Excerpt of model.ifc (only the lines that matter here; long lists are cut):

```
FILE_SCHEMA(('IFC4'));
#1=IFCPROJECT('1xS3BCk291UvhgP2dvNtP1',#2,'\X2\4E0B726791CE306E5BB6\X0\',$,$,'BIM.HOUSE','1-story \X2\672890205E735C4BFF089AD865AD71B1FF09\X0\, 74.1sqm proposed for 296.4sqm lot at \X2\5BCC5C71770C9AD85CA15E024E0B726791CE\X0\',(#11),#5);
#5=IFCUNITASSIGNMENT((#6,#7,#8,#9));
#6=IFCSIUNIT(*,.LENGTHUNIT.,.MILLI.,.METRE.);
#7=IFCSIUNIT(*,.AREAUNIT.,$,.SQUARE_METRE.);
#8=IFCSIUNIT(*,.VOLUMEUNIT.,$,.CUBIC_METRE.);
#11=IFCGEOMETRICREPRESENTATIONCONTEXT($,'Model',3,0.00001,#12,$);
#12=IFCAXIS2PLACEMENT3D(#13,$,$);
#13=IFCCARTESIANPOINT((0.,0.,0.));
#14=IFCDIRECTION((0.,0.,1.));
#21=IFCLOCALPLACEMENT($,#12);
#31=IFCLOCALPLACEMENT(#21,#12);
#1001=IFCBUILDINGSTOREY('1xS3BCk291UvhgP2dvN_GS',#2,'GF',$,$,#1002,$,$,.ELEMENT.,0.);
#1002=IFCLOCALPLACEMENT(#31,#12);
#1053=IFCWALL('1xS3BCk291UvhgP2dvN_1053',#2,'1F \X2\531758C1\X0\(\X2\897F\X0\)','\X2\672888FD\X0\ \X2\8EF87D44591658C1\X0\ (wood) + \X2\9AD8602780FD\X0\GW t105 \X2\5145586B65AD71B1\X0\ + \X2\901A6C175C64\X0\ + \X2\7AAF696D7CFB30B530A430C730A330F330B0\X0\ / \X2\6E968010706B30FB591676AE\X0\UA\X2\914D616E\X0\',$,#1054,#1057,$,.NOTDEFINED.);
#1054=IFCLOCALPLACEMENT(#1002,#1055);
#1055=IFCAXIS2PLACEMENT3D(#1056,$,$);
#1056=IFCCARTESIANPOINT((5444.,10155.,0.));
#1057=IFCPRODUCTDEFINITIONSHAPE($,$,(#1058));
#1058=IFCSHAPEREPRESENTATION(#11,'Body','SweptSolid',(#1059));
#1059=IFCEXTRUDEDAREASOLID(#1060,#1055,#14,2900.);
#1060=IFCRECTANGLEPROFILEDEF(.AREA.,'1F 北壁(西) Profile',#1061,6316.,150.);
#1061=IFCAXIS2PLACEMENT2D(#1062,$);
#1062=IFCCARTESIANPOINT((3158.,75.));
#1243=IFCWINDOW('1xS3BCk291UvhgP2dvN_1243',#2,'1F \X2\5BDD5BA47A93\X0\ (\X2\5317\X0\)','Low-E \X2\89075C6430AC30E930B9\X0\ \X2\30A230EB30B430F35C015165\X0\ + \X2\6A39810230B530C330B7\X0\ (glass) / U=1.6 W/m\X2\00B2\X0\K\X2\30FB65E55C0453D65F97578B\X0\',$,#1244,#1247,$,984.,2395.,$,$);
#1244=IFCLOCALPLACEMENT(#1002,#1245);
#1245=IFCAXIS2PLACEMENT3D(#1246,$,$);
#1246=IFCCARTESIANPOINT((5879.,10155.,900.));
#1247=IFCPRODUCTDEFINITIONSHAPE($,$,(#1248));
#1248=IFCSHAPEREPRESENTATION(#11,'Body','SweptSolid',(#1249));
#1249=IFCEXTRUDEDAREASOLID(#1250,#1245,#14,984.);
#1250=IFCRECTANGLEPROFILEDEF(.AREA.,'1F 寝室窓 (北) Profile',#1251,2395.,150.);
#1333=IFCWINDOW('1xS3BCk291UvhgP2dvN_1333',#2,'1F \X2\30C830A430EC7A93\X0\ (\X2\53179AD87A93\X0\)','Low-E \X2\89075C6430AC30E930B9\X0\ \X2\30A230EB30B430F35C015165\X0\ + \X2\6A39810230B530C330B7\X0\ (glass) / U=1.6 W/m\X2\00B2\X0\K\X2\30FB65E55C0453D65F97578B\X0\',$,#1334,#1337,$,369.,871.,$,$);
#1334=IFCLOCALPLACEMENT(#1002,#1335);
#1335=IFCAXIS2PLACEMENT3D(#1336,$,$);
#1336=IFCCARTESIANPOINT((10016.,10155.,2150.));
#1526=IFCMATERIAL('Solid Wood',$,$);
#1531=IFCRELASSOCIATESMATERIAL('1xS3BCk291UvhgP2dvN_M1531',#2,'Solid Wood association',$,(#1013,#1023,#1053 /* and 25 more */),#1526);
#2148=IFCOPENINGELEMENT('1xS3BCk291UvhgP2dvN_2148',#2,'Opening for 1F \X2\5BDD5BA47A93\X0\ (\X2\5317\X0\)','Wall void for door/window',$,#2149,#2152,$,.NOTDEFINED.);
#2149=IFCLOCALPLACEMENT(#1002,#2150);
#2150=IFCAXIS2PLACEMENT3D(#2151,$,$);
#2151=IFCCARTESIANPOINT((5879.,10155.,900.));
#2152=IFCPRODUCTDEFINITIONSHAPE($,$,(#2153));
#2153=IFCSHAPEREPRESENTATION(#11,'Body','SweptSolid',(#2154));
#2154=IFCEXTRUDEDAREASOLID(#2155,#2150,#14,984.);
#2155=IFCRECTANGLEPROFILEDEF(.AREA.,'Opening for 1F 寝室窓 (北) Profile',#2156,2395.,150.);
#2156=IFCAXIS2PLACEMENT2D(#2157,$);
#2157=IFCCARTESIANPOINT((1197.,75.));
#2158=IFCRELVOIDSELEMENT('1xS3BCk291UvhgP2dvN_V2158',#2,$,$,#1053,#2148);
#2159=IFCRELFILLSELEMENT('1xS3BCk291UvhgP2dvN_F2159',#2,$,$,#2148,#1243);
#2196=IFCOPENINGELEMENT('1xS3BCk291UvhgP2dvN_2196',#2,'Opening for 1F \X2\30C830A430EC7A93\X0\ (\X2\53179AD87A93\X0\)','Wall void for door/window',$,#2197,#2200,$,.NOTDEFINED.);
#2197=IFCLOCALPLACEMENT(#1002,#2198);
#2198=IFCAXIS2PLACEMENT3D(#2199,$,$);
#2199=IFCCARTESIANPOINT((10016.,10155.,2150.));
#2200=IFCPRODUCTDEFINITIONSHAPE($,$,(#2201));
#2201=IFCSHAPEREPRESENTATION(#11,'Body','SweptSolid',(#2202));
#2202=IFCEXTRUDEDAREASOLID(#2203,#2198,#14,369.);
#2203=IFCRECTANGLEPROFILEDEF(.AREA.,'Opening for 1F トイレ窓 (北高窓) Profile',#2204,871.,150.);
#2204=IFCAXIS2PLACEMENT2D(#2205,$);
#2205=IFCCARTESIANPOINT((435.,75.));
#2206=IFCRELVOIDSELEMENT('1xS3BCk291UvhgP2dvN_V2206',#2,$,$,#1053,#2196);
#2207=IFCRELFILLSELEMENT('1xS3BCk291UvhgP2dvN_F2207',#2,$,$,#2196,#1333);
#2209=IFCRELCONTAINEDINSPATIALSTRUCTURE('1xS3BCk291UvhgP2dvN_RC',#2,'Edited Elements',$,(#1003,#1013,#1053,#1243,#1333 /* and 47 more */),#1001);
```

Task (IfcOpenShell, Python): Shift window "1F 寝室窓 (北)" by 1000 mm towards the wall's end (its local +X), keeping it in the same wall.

```python
import ifcopenshell
import ifcopenshell.api.geometry
import ifcopenshell.util.placement

model = ifcopenshell.open("model.ifc")

window = model.by_guid("1xS3BCk291UvhgP2dvN_1243")
opening = window.FillsVoids[0].RelatingOpeningElement
wall = opening.VoidsElements[0].RelatingBuildingElement

wall_matrix = ifcopenshell.util.placement.get_local_placement(wall.ObjectPlacement)
shift = wall_matrix[:3, 0] * 1000.0
before = ifcopenshell.util.placement.get_local_placement(window.ObjectPlacement)[:3, 3].copy()

# The window is not placed relative to its opening, so move both.
for product in (opening, window):
    matrix = ifcopenshell.util.placement.get_local_placement(product.ObjectPlacement)
    matrix[:3, 3] += shift
    ifcopenshell.api.geometry.edit_object_placement(model, product=product, matrix=matrix, is_si=False)

after = ifcopenshell.util.placement.get_local_placement(window.ObjectPlacement)[:3, 3]
print("window moved by", (after - before).round(3) + 0.0)

model.write("model_updated.ifc")
```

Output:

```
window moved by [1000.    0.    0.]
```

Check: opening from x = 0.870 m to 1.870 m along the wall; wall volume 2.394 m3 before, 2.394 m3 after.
